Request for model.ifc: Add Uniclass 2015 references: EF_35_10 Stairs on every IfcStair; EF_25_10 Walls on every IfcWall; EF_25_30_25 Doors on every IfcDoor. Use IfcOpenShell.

First a look at what the model holds.

```python
import ifcopenshell

model = ifcopenshell.open("model.ifc")
print(model.schema)
print("classifications:", [c.Name for c in model.by_type("IfcClassification")])
for ifc_class in ("IfcDoor", "IfcRoof", "IfcStair", "IfcWall", "IfcWindow"):
    print(ifc_class, len(model.by_type(ifc_class)))
```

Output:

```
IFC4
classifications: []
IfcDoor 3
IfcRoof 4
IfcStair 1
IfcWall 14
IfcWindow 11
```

```python
import ifcopenshell
import ifcopenshell.api.classification

model = ifcopenshell.open("model.ifc")

system = ifcopenshell.api.classification.add_classification(model, classification="Uniclass 2015")

codes = {
    "IfcStair": ("EF_35_10", "Stairs"),
    "IfcWall": ("EF_25_10", "Walls"),
    "IfcDoor": ("EF_25_30_25", "Doors"),
}
for ifc_class, (code, name) in codes.items():
    products = model.by_type(ifc_class)
    ifcopenshell.api.classification.add_reference(
        model, products=products, classification=system, identification=code, name=name
    )
    print(code, len(products))

model.write("model_rev.ifc")
```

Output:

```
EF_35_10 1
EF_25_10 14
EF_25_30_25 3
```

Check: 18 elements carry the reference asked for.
